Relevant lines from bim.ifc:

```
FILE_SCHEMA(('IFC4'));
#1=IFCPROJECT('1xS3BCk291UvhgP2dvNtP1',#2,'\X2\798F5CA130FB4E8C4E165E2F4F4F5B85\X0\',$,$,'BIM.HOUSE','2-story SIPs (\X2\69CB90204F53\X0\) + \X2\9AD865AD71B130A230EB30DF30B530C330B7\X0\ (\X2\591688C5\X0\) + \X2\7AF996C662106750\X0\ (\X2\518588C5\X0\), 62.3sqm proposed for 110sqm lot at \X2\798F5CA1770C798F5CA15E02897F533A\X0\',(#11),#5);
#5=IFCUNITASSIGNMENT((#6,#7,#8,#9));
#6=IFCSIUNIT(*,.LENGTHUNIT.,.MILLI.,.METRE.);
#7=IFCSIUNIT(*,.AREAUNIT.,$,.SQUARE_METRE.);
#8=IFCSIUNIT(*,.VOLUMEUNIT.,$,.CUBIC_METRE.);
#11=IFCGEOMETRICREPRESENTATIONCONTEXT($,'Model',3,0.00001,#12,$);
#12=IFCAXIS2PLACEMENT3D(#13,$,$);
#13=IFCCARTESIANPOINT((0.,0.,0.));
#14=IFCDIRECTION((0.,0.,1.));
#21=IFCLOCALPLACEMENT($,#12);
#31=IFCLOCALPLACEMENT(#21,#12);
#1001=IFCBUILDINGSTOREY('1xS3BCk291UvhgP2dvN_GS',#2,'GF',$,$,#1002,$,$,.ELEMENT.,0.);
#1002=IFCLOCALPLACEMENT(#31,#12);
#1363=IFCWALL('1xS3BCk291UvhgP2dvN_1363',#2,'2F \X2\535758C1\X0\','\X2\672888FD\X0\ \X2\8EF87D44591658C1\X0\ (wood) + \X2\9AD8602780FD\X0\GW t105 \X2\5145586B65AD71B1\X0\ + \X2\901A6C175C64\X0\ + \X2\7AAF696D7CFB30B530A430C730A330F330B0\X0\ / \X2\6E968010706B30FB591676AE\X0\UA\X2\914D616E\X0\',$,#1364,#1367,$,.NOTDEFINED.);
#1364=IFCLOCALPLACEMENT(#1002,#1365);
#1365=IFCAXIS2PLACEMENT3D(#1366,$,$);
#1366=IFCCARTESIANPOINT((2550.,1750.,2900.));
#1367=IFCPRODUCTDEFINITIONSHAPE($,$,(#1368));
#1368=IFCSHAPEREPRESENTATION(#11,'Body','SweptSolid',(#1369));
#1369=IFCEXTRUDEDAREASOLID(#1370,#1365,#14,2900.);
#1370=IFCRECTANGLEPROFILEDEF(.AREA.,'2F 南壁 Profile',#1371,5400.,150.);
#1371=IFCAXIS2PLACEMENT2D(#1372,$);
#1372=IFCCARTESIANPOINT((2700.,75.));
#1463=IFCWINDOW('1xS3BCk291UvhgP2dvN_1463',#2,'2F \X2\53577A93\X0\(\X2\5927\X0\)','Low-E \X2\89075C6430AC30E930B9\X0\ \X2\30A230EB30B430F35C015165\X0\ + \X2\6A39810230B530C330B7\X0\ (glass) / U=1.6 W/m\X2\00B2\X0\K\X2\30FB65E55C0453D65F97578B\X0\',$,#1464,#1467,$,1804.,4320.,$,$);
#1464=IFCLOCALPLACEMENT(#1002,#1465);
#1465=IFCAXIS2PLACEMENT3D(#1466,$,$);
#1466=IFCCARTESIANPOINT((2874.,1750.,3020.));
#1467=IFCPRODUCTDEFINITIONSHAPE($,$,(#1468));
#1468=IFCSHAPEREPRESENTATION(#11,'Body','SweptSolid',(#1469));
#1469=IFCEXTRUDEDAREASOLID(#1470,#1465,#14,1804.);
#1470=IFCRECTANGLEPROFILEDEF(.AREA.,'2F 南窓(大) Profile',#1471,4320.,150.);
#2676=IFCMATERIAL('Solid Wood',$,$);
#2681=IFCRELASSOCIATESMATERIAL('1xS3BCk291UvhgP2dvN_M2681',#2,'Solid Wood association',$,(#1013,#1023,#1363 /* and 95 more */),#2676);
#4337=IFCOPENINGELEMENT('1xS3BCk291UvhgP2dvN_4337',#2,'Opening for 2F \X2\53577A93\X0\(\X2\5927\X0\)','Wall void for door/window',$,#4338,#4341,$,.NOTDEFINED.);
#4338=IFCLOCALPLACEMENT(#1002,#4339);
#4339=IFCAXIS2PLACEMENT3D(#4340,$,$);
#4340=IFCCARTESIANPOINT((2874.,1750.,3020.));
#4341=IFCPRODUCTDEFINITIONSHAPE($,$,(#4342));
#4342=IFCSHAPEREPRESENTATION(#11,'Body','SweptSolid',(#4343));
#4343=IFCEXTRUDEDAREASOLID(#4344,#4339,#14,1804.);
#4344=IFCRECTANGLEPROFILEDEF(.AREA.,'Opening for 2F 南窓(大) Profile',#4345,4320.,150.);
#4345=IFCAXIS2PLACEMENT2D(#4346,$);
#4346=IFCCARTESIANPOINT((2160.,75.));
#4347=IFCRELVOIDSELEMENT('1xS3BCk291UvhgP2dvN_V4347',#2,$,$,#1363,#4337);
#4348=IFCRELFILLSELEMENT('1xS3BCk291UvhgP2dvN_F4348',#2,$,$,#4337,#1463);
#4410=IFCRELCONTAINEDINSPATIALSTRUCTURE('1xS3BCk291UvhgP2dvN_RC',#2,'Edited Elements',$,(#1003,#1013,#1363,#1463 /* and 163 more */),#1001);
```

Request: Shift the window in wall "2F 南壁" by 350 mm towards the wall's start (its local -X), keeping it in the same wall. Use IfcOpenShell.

```python
import ifcopenshell
import ifcopenshell.api.geometry
import ifcopenshell.util.placement
import ifcopenshell.util.unit

model = ifcopenshell.open("bim.ifc")
unit_scale = ifcopenshell.util.unit.calculate_unit_scale(model)

window = model.by_guid("1xS3BCk291UvhgP2dvN_1463")
opening = window.FillsVoids[0].RelatingOpeningElement
wall = opening.VoidsElements[0].RelatingBuildingElement

wall_matrix = ifcopenshell.util.placement.get_local_placement(wall.ObjectPlacement)
shift = wall_matrix[:3, 0] * -0.35 / unit_scale
before = ifcopenshell.util.placement.get_local_placement(window.ObjectPlacement)[:3, 3].copy()

# The window is not placed relative to its opening, so move both.
for product in (opening, window):
    matrix = ifcopenshell.util.placement.get_local_placement(product.ObjectPlacement)
    matrix[:3, 3] += shift
    ifcopenshell.api.geometry.edit_object_placement(model, product=product, matrix=matrix, is_si=False)

after = ifcopenshell.util.placement.get_local_placement(window.ObjectPlacement)[:3, 3]
print("window moved by", (after - before).round(3) + 0.0)

model.write("bim_rev.ifc")
```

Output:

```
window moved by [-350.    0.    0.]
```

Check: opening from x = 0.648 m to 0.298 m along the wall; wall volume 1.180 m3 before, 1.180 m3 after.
